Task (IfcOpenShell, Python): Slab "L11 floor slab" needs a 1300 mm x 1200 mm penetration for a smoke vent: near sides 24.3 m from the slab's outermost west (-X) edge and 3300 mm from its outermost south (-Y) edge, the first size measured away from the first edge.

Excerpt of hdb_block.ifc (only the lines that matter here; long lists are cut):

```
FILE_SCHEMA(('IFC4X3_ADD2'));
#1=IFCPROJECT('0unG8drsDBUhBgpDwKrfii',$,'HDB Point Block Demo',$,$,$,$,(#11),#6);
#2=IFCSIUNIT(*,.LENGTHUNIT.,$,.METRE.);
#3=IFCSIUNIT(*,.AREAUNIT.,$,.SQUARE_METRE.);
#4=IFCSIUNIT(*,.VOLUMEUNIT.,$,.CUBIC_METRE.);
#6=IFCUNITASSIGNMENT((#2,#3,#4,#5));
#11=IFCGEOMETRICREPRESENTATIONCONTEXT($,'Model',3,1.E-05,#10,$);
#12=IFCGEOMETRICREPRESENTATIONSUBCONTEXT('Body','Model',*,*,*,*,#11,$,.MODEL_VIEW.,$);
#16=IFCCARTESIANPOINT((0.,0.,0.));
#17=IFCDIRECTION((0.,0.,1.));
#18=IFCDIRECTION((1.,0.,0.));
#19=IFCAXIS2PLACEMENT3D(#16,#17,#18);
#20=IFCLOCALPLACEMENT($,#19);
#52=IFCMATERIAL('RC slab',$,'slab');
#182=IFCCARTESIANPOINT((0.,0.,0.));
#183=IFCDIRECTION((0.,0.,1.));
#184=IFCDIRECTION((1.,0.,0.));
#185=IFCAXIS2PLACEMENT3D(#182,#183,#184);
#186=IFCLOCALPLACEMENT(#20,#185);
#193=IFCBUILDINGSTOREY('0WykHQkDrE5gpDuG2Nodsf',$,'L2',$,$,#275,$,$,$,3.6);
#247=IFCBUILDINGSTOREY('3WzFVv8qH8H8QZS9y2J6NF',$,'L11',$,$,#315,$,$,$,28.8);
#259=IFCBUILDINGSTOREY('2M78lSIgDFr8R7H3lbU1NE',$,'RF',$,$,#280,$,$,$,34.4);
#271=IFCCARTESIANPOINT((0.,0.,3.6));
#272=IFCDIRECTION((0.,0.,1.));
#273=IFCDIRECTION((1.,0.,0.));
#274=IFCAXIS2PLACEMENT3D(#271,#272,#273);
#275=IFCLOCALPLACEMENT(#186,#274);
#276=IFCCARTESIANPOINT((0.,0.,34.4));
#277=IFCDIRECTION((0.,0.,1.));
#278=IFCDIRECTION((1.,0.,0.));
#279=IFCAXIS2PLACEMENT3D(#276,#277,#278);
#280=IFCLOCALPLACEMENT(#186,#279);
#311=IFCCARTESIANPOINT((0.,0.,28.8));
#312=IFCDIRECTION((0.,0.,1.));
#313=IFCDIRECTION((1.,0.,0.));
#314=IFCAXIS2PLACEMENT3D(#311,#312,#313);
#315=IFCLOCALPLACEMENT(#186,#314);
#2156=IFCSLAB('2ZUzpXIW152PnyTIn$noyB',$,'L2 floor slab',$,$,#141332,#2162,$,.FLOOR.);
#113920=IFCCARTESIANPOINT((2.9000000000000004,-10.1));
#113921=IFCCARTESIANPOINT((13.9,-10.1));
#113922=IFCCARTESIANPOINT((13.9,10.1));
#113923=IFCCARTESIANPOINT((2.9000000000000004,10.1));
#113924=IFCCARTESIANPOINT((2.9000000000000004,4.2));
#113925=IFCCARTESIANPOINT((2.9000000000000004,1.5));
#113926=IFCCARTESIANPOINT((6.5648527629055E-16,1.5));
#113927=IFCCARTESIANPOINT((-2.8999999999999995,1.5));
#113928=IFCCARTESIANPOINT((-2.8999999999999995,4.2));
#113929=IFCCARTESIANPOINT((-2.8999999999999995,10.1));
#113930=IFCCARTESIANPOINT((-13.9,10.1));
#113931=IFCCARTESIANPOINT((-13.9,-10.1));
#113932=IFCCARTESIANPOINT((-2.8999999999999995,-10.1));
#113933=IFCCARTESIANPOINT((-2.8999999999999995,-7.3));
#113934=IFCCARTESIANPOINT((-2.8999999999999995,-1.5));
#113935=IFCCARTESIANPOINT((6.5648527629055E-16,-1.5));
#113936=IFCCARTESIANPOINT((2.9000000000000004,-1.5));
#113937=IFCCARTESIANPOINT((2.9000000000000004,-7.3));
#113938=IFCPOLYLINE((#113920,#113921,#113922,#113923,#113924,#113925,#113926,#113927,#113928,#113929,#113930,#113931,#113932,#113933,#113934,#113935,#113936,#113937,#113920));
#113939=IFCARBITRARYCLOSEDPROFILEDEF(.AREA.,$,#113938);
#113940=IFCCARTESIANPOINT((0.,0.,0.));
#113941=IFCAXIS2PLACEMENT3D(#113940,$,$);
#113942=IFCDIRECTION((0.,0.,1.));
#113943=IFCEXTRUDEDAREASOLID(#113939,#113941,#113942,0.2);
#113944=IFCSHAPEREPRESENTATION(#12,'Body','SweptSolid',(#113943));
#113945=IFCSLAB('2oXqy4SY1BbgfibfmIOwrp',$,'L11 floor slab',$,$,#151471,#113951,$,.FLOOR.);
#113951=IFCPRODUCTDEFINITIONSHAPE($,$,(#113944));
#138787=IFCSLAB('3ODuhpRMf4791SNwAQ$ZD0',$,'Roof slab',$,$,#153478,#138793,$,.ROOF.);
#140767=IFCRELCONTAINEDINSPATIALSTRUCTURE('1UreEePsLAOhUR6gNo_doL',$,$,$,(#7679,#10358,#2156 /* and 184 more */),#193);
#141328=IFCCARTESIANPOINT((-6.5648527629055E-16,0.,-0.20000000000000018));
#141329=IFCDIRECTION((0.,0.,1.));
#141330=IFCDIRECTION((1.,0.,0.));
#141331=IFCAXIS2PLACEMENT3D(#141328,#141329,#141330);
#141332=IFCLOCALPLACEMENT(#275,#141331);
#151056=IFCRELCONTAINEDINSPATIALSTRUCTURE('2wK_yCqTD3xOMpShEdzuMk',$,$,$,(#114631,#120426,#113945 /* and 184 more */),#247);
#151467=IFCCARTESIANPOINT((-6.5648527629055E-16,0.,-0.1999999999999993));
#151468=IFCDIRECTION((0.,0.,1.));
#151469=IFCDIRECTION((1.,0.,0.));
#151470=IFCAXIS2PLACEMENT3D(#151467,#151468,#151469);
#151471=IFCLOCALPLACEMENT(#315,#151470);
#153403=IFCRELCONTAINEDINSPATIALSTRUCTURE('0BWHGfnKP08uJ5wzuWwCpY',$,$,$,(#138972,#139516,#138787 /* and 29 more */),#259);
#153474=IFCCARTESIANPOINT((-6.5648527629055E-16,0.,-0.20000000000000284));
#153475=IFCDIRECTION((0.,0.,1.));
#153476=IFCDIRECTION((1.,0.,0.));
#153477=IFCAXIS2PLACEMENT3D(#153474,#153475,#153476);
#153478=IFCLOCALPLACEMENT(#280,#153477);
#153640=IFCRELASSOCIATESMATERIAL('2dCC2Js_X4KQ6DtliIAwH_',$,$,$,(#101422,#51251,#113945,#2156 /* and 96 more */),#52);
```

```python
import numpy as np
import ifcopenshell
import ifcopenshell.api.feature
import ifcopenshell.api.geometry
import ifcopenshell.api.root
import ifcopenshell.geom
import ifcopenshell.util.placement
import ifcopenshell.util.representation
import ifcopenshell.util.shape
import ifcopenshell.util.unit

model = ifcopenshell.open("hdb_block.ifc")
unit_scale = ifcopenshell.util.unit.calculate_unit_scale(model)
settings = ifcopenshell.geom.settings()


def volume(element):
    """Net volume in cubic metres, openings subtracted."""
    shape = ifcopenshell.geom.create_shape(settings, element)
    return ifcopenshell.util.shape.get_volume(shape.geometry)


slab = model.by_guid("2oXqy4SY1BbgfibfmIOwrp")
before = volume(slab)

# Extent in the slab's own axes, in metres. The edges named are its -X and -Y sides.
slab_shape = ifcopenshell.geom.create_shape(settings, slab)
vertices = ifcopenshell.util.shape.get_vertices(slab_shape.geometry)
x_min, y_min, bottom = vertices.min(axis=0)
top = vertices[:, 2].max()

opening = ifcopenshell.api.root.create_entity(model, ifc_class="IfcOpeningElement", name="Smoke vent opening", predefined_type="OPENING")
context = ifcopenshell.util.representation.get_context(model, "Model", "Body", "MODEL_VIEW")
width, depth = 1.3, 1.2
outline = [(0.0, 0.0), (width, 0.0), (width, depth), (0.0, depth), (0.0, 0.0)]
# Overshoot both faces by 50 mm so the cut is clean.
shape = ifcopenshell.api.geometry.add_slab_representation(
    model, context=context, depth=top - bottom + 0.1, polyline=outline
)
ifcopenshell.api.geometry.assign_representation(model, product=opening, representation=shape)

matrix = ifcopenshell.util.placement.get_local_placement(slab.ObjectPlacement)
matrix[:, 3] = matrix @ np.append(np.array([x_min + 24.3, y_min + 3.3, bottom - 0.05]) / unit_scale, 1.0)
ifcopenshell.api.geometry.edit_object_placement(model, product=opening, matrix=matrix, is_si=False)
ifcopenshell.api.feature.add_feature(model, feature=opening, element=slab)

after = volume(slab)

print(f"slab volume {before:.3f} -> {after:.3f} m3")

model.write("hdb_block_v2.ifc")
```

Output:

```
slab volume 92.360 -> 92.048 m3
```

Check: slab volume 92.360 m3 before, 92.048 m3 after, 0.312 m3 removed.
